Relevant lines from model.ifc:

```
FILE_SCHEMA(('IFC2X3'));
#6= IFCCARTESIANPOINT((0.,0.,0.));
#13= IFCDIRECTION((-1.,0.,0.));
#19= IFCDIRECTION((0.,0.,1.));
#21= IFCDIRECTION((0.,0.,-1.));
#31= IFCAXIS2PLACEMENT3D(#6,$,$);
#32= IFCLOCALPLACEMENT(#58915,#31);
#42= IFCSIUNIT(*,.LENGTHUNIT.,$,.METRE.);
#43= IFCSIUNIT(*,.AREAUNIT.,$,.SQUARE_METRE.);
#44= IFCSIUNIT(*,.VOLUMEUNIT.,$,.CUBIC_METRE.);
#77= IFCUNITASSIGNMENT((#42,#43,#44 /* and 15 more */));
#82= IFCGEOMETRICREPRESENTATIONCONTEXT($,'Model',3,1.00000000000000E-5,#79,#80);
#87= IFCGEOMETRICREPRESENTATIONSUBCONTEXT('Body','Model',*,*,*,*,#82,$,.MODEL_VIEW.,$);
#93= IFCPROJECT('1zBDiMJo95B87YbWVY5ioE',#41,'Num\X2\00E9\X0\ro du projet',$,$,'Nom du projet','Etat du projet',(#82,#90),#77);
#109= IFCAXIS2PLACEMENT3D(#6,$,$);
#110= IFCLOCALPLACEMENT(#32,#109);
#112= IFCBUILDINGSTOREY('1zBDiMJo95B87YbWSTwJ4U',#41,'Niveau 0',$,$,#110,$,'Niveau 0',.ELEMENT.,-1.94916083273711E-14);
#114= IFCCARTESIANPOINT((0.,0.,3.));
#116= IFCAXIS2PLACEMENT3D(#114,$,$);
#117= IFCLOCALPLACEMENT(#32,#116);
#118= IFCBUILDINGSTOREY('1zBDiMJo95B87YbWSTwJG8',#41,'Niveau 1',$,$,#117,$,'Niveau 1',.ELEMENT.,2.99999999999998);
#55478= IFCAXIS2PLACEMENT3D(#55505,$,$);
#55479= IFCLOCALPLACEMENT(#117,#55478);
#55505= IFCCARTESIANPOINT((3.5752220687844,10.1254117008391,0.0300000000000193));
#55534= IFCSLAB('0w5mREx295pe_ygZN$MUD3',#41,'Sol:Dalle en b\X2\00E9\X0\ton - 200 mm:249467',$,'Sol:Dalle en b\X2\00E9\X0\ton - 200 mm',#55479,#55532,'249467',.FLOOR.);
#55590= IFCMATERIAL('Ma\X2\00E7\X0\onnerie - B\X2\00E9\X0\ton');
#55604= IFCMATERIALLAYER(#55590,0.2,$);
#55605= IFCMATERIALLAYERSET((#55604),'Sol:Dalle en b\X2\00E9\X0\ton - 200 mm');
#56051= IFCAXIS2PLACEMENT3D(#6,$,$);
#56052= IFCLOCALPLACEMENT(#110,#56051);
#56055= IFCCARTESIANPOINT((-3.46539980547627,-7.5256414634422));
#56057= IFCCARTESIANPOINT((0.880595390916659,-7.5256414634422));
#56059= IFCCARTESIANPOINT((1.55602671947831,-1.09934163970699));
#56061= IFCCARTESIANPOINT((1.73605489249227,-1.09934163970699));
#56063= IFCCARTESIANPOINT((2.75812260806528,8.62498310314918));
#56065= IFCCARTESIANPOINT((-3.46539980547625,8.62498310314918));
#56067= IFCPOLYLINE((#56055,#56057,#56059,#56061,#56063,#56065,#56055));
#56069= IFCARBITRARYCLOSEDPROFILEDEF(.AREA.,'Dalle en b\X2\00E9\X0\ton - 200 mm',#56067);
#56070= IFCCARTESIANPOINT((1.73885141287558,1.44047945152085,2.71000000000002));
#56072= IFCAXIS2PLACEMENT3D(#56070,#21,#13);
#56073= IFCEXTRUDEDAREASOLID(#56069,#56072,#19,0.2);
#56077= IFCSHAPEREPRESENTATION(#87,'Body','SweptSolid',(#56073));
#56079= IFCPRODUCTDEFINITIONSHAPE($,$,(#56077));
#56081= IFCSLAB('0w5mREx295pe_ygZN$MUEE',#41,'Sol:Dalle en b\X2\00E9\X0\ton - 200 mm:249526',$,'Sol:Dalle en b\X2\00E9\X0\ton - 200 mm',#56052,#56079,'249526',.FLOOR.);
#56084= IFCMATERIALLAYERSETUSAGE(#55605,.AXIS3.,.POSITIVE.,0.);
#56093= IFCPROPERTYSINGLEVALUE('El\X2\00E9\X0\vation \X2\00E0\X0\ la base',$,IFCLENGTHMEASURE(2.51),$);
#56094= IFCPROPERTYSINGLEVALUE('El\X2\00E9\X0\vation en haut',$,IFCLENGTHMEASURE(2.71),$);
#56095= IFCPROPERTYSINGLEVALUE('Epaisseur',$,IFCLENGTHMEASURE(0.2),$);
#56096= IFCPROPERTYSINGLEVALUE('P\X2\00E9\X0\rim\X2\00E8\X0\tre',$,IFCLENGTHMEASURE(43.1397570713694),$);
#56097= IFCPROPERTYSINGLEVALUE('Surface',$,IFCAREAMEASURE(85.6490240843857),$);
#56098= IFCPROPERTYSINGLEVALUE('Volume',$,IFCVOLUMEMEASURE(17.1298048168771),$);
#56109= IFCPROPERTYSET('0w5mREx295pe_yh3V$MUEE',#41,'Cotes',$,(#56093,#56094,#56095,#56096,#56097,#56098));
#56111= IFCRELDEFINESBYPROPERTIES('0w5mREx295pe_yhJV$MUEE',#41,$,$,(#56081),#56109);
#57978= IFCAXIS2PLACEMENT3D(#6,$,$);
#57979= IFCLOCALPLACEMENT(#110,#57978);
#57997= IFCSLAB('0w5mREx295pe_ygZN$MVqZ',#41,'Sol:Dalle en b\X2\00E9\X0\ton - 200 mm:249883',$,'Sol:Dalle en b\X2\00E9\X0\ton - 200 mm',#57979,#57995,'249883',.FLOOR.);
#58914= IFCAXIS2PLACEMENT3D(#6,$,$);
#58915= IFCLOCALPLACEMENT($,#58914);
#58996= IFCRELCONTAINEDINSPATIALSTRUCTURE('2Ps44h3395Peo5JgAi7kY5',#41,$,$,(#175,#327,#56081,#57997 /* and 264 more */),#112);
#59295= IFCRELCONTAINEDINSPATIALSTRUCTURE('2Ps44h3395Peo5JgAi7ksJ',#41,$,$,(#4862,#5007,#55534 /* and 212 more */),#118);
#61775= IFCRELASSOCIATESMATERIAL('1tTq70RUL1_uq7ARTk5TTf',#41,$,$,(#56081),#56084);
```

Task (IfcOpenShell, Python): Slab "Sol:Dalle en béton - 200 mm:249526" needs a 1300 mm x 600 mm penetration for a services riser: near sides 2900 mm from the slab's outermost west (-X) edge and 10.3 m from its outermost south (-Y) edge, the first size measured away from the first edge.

```python
import numpy as np
import ifcopenshell
import ifcopenshell.api.feature
import ifcopenshell.api.geometry
import ifcopenshell.api.pset
import ifcopenshell.api.root
import ifcopenshell.geom
import ifcopenshell.util.element
import ifcopenshell.util.placement
import ifcopenshell.util.representation
import ifcopenshell.util.shape
import ifcopenshell.util.unit

model = ifcopenshell.open("model.ifc")
unit_scale = ifcopenshell.util.unit.calculate_unit_scale(model)
area_scale = ifcopenshell.util.unit.calculate_unit_scale(model, "AREAUNIT")
volume_scale = ifcopenshell.util.unit.calculate_unit_scale(model, "VOLUMEUNIT")
settings = ifcopenshell.geom.settings()


def volume(element):
    """Net volume in cubic metres, openings subtracted."""
    shape = ifcopenshell.geom.create_shape(settings, element)
    return ifcopenshell.util.shape.get_volume(shape.geometry)


slab = model.by_guid("0w5mREx295pe_ygZN$MUEE")
before = volume(slab)

# Extent in the slab's own axes, in metres. The edges named are its -X and -Y sides.
slab_shape = ifcopenshell.geom.create_shape(settings, slab)
vertices = ifcopenshell.util.shape.get_vertices(slab_shape.geometry)
x_min, y_min, bottom = vertices.min(axis=0)
top = vertices[:, 2].max()

opening = ifcopenshell.api.root.create_entity(model, ifc_class="IfcOpeningElement", name="Services riser opening")
context = ifcopenshell.util.representation.get_context(model, "Model", "Body", "MODEL_VIEW")
width, depth = 1.3, 0.6
outline = [(0.0, 0.0), (width, 0.0), (width, depth), (0.0, depth), (0.0, 0.0)]
# Overshoot both faces by 50 mm so the cut is clean.
shape = ifcopenshell.api.geometry.add_slab_representation(
    model, context=context, depth=top - bottom + 0.1, polyline=outline
)
ifcopenshell.api.geometry.assign_representation(model, product=opening, representation=shape)

matrix = ifcopenshell.util.placement.get_local_placement(slab.ObjectPlacement)
matrix[:, 3] = matrix @ np.append(np.array([x_min + 2.9, y_min + 10.3, bottom - 0.05]) / unit_scale, 1.0)
ifcopenshell.api.geometry.edit_object_placement(model, product=opening, matrix=matrix, is_si=False)
ifcopenshell.api.feature.add_feature(model, feature=opening, element=slab)

after = volume(slab)

# Update the slab's stored quantities.
pset = model.by_id(ifcopenshell.util.element.get_pset(slab, "Cotes", should_inherit=False)["id"])
ifcopenshell.api.pset.edit_pset(model, pset=pset, properties={
    "Surface": model.create_entity("IfcAreaMeasure", after / (top - bottom) / area_scale),
    "Volume": model.create_entity("IfcVolumeMeasure", after / volume_scale),
})

print(f"slab volume {before:.3f} -> {after:.3f} m3")

model.write("model_edited.ifc")
```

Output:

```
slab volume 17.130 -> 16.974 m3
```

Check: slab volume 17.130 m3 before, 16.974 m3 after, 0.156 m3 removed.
